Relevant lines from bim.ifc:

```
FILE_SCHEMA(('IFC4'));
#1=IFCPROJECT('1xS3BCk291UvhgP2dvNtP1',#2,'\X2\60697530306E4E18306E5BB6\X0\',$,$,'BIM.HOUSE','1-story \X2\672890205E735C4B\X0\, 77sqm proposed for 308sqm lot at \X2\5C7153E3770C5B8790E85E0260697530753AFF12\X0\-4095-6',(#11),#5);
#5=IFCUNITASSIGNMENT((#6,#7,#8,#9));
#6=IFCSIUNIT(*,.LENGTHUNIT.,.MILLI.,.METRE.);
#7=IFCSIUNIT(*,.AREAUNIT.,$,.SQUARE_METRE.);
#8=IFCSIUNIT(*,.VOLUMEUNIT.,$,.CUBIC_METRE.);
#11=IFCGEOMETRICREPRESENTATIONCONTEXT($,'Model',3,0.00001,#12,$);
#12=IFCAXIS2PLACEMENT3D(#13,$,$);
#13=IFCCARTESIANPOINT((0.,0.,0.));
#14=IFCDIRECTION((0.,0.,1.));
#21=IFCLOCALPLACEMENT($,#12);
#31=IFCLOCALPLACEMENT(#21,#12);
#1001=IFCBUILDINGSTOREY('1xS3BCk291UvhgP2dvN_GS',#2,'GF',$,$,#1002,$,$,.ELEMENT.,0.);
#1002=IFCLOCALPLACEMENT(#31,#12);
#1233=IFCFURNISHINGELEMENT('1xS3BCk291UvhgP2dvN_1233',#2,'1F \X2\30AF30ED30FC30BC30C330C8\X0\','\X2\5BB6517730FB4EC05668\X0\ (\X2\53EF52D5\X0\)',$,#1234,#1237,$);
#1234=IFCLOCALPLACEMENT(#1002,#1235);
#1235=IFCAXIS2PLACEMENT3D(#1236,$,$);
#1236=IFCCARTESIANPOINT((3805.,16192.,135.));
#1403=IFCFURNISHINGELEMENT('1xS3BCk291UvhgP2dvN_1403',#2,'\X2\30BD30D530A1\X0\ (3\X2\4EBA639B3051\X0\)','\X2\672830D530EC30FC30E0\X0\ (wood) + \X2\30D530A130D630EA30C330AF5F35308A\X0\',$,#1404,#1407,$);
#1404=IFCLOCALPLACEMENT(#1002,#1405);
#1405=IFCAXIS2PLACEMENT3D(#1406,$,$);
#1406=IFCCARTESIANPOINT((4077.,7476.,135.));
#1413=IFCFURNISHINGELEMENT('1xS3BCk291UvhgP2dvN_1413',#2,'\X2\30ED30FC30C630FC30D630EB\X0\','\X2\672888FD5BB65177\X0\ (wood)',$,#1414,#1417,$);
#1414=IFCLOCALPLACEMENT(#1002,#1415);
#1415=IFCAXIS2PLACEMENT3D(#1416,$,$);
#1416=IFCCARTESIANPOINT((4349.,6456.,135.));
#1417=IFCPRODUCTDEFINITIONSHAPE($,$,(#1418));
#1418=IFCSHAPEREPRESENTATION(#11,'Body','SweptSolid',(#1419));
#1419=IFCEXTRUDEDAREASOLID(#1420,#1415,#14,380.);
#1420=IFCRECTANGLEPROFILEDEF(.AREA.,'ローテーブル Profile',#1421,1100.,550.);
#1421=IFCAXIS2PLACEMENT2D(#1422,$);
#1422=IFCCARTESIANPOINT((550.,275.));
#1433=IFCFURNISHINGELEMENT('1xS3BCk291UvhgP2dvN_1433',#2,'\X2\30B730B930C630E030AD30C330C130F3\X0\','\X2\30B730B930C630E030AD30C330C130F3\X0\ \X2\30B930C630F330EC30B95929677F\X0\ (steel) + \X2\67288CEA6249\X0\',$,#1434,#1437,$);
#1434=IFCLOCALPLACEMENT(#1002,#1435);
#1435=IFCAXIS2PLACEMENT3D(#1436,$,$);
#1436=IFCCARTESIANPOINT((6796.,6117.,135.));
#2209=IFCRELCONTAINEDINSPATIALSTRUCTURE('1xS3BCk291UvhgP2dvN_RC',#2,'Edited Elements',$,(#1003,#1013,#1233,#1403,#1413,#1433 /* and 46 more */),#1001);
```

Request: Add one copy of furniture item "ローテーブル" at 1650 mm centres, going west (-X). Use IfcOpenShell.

```python
import numpy as np
import ifcopenshell
import ifcopenshell.api.geometry
import ifcopenshell.api.root
import ifcopenshell.util.element
import ifcopenshell.util.placement
import ifcopenshell.util.unit

model = ifcopenshell.open("bim.ifc")
unit_scale = ifcopenshell.util.unit.calculate_unit_scale(model)


def reuse_history(source, copy):
    """copy_class also copies each property set's owner history, people and application; keep the originals."""
    for rel in copy.IsDefinedBy:
        if rel.is_a("IfcRelDefinesByProperties") and (history := rel.RelatingPropertyDefinition.OwnerHistory):
            rel.RelatingPropertyDefinition.OwnerHistory = source.OwnerHistory
            ifcopenshell.util.element.remove_deep2(model, history)


source = model.by_guid("1xS3BCk291UvhgP2dvN_1413")
base = ifcopenshell.util.placement.get_local_placement(source.ObjectPlacement)
step = np.array([-1.0, 0.0, 0.0]) * 1.65 / unit_scale

for i in range(1, 2):
    copy = ifcopenshell.api.root.copy_class(model, product=source)
    copy.Representation = ifcopenshell.util.element.copy_deep(
        model, source.Representation, exclude=["IfcGeometricRepresentationContext", "IfcRepresentationMap"]
    )
    reuse_history(source, copy)
    matrix = base.copy()
    matrix[:3, 3] += i * step
    print("added at", matrix[:3, 3].round(3) + 0.0)
    ifcopenshell.api.geometry.edit_object_placement(model, product=copy, matrix=matrix, is_si=False)

model.write("bim_updated.ifc")
```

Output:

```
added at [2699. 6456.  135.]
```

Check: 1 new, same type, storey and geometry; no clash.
